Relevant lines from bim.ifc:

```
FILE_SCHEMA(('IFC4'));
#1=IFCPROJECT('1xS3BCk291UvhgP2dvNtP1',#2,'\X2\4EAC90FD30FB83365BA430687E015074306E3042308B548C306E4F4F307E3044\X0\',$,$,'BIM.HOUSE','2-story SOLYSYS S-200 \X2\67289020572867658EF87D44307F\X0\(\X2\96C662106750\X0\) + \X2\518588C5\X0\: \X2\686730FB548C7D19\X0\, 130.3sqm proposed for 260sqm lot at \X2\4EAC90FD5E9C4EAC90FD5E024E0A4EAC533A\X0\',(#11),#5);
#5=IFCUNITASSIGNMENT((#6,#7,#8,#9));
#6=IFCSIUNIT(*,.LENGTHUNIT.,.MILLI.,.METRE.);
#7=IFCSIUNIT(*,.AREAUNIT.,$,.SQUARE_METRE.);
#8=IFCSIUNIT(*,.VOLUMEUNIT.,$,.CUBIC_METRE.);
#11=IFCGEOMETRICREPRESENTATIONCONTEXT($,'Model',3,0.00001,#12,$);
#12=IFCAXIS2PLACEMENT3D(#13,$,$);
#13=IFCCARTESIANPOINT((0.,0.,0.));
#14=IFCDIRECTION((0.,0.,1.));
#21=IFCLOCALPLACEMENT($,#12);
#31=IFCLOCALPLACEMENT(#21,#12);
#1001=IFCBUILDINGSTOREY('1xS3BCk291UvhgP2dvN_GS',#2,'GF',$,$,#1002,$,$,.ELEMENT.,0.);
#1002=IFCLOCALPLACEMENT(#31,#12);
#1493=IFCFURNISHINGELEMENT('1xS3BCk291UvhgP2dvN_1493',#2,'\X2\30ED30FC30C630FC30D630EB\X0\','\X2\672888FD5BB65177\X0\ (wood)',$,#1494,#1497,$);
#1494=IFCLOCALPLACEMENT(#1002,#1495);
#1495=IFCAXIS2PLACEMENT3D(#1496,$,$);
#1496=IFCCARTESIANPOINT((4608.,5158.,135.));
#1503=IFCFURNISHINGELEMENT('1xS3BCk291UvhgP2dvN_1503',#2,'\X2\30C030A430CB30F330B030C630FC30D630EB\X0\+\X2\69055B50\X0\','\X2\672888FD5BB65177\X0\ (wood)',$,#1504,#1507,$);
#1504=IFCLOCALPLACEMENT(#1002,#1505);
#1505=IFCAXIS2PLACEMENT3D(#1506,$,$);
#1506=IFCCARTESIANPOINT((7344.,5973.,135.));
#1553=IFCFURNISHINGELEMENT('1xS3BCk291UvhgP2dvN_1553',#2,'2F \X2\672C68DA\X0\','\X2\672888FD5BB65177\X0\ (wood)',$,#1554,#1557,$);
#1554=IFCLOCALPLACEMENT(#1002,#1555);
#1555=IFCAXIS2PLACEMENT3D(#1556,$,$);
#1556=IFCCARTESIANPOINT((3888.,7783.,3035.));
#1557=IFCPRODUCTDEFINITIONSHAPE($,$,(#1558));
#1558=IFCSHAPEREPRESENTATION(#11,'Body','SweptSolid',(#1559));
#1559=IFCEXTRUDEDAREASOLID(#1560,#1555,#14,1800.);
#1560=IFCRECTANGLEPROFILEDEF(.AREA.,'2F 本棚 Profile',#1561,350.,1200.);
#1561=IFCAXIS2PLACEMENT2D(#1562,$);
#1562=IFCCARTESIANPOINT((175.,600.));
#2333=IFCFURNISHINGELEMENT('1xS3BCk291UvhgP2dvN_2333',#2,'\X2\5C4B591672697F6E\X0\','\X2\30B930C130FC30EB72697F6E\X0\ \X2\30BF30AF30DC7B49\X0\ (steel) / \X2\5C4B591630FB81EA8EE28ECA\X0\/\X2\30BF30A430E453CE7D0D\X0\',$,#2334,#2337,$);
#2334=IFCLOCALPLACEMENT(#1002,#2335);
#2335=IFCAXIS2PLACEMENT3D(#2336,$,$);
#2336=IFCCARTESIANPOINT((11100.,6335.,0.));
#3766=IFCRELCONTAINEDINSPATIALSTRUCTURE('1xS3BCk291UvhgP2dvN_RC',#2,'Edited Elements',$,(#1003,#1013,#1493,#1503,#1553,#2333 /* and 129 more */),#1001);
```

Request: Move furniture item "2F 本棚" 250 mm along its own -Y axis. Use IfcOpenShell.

```python
import ifcopenshell
import ifcopenshell.api.geometry
import ifcopenshell.util.placement
import ifcopenshell.util.unit

model = ifcopenshell.open("bim.ifc")
unit_scale = ifcopenshell.util.unit.calculate_unit_scale(model)

item = model.by_id(1553)
matrix = ifcopenshell.util.placement.get_local_placement(item.ObjectPlacement)
matrix[:3, 3] -= matrix[:3, 1] * 0.25 / unit_scale
ifcopenshell.api.geometry.edit_object_placement(model, product=item, matrix=matrix, is_si=False)

print(ifcopenshell.util.placement.get_local_placement(item.ObjectPlacement).round(3) + 0.0)

model.write("bim_edited.ifc")
```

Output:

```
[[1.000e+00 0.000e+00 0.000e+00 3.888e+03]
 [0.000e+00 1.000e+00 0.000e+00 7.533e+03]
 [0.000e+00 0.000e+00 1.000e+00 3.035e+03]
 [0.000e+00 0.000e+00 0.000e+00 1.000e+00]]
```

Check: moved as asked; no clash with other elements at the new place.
